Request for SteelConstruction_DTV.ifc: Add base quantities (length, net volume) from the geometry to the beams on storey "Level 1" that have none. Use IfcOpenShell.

First a look at what the model holds.

```python
import ifcopenshell
import ifcopenshell.util.element
import ifcopenshell.util.unit

model = ifcopenshell.open("SteelConstruction_DTV.ifc")
print(model.schema)
for unit_type in ("LENGTHUNIT", "AREAUNIT", "VOLUMEUNIT"):
    print(unit_type, ifcopenshell.util.unit.calculate_unit_scale(model, unit_type))
storey = next(s for s in model.by_type("IfcBuildingStorey") if s.Name == "Level 1")
beams = [e for e in ifcopenshell.util.element.get_decomposition(storey) if e.is_a("IfcBeam")]
for e in sorted(beams, key=lambda e: e.id()):
    print(e.id(), e.is_a(), e.Name, list(ifcopenshell.util.element.get_psets(e, qtos_only=True)), sep=" | ")
```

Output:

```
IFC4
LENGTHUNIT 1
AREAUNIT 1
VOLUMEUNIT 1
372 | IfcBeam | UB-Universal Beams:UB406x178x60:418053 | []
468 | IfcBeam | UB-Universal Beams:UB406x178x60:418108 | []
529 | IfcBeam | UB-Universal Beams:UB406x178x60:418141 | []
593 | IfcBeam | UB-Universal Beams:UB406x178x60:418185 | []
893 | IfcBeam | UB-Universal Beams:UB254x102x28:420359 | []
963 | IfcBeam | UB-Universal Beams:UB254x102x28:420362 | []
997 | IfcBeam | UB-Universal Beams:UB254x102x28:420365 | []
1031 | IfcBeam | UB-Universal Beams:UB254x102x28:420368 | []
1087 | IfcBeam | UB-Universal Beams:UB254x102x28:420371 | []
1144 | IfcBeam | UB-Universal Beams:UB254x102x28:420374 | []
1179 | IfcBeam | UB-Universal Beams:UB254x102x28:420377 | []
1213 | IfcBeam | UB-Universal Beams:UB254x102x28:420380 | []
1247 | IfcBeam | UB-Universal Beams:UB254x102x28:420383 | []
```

```python
import ifcopenshell
import ifcopenshell.api.pset
import ifcopenshell.geom
import ifcopenshell.util.element
import ifcopenshell.util.shape
import ifcopenshell.util.unit

model = ifcopenshell.open("SteelConstruction_DTV.ifc")
unit_scale = ifcopenshell.util.unit.calculate_unit_scale(model)
volume_scale = ifcopenshell.util.unit.calculate_unit_scale(model, "VOLUMEUNIT")
settings = ifcopenshell.geom.settings()

storey = next(s for s in model.by_type("IfcBuildingStorey") if s.Name == "Level 1")
beams = [e for e in ifcopenshell.util.element.get_decomposition(storey) if e.is_a("IfcBeam")]

for e in sorted(beams, key=lambda e: e.id()):
    if ifcopenshell.util.element.get_psets(e, qtos_only=True, should_inherit=False):
        continue
    # Geometry comes back in metres, in the element's own axes.
    shape = ifcopenshell.geom.create_shape(settings, e)
    values = {
        "Length": ifcopenshell.util.shape.get_max_xyz(shape.geometry) / unit_scale,
        "NetVolume": ifcopenshell.util.shape.get_volume(shape.geometry) / volume_scale,
    }
    qto = ifcopenshell.api.pset.add_qto(model, product=e, name="Qto_BeamBaseQuantities")
    ifcopenshell.api.pset.edit_qto(model, qto=qto, properties=values)
    print(e.id(), {k: round(v, 3) for k, v in values.items()})

model.write("SteelConstruction_DTV-out.ifc")
```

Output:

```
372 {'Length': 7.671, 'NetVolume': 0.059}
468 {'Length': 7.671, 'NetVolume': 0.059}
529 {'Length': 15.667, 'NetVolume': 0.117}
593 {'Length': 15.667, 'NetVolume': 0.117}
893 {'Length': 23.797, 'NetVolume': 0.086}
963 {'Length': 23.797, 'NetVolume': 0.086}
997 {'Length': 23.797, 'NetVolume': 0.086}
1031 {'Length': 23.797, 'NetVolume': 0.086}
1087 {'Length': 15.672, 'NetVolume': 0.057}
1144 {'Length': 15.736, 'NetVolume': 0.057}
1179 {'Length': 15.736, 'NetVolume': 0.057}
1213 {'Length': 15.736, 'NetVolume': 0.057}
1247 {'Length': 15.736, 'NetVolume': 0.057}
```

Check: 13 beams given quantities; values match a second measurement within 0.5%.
